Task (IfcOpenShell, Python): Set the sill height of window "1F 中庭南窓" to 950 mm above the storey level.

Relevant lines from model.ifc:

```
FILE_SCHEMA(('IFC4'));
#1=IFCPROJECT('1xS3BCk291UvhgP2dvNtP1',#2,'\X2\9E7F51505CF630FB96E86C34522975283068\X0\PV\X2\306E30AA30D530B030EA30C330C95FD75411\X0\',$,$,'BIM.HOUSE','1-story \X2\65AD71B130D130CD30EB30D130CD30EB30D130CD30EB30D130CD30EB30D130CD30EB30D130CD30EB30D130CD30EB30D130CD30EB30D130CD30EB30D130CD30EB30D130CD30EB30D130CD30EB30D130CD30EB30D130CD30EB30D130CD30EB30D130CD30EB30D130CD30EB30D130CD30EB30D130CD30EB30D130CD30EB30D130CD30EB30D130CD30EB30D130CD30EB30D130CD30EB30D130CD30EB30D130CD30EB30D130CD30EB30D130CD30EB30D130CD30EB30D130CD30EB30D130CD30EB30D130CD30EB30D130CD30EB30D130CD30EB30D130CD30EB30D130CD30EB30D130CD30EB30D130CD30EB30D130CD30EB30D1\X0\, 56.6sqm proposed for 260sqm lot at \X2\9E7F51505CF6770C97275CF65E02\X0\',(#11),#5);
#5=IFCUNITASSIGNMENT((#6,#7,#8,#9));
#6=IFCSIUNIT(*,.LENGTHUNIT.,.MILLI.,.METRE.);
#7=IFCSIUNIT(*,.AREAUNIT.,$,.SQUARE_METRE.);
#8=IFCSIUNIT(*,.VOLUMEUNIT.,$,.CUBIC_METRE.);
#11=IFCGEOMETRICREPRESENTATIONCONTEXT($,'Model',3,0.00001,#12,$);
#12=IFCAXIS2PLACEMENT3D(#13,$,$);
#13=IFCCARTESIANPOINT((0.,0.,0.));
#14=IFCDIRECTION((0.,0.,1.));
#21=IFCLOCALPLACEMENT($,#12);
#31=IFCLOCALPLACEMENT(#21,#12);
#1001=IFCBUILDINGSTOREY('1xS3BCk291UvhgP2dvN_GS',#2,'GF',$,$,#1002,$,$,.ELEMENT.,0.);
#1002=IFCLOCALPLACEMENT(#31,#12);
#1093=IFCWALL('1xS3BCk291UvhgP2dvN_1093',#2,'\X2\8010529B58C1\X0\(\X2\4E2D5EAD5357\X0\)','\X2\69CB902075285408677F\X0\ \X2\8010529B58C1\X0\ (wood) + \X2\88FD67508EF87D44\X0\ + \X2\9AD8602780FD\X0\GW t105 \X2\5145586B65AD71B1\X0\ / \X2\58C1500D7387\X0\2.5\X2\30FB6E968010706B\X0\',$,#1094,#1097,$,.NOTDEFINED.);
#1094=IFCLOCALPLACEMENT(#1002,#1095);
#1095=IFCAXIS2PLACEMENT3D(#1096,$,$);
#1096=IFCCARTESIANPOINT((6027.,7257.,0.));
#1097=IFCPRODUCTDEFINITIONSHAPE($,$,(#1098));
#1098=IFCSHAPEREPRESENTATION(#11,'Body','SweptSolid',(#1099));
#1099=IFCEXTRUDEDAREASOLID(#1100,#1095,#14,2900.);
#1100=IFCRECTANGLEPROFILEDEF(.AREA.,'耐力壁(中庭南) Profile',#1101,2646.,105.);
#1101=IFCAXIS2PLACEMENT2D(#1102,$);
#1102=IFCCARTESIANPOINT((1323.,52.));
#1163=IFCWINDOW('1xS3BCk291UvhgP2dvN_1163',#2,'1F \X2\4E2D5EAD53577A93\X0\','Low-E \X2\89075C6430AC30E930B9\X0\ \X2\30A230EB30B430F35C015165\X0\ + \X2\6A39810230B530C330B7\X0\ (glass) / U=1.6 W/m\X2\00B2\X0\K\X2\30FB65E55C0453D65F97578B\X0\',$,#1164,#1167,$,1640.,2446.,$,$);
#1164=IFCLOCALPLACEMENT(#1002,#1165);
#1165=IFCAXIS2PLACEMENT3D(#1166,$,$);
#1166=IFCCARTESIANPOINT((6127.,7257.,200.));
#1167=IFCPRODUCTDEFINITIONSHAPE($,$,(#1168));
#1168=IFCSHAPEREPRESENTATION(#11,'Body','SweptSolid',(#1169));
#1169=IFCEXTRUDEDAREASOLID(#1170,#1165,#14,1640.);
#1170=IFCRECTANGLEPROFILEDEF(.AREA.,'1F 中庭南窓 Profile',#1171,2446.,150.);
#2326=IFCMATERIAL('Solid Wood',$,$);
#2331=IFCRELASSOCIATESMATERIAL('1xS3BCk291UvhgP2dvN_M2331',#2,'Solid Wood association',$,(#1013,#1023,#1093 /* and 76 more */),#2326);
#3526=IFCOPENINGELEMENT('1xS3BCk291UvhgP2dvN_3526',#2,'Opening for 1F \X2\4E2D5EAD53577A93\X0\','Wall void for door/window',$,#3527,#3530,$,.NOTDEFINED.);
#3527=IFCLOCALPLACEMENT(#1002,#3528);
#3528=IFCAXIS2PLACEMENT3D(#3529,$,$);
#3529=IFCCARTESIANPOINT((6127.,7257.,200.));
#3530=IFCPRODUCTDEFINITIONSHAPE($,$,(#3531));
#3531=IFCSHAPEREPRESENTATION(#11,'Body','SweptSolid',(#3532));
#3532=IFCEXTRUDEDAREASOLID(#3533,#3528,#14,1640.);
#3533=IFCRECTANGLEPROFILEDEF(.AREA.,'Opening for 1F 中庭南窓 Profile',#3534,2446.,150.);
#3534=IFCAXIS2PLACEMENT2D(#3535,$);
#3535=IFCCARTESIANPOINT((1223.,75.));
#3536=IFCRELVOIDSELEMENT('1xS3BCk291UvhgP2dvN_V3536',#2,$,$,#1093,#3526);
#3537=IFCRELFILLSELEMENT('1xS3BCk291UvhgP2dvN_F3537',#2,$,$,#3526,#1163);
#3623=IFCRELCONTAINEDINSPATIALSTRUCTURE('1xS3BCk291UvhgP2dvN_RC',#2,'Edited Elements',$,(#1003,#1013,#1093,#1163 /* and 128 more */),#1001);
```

```python
import numpy as np
import ifcopenshell
import ifcopenshell.api.geometry
import ifcopenshell.geom
import ifcopenshell.util.element
import ifcopenshell.util.placement
import ifcopenshell.util.shape
import ifcopenshell.util.unit

model = ifcopenshell.open("model.ifc")
unit_scale = ifcopenshell.util.unit.calculate_unit_scale(model)

window = model.by_id(1163)
opening = window.FillsVoids[0].RelatingOpeningElement
storey = ifcopenshell.util.element.get_container(window, ifc_class="IfcBuildingStorey")
level = ifcopenshell.util.placement.get_local_placement(storey.ObjectPlacement)[2, 3]

# The opening's origin need not be at the sill, so measure its lowest point.
shape = ifcopenshell.geom.create_shape(ifcopenshell.geom.settings(), opening)
bottom = ifcopenshell.util.shape.get_shape_bottom_elevation(shape, shape.geometry) / unit_scale
dz = level + 0.95 / unit_scale - bottom

shift = np.array([0.0, 0.0, dz])
# The window is not placed relative to its opening, so move both.
for product in (opening, window):
    matrix = ifcopenshell.util.placement.get_local_placement(product.ObjectPlacement)
    matrix[:3, 3] += shift
    ifcopenshell.api.geometry.edit_object_placement(model, product=product, matrix=matrix, is_si=False)

print(f"moved by {dz * unit_scale:+.3f} m")

model.write("model_v2.ifc")
```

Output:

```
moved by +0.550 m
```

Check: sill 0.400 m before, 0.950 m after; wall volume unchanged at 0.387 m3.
